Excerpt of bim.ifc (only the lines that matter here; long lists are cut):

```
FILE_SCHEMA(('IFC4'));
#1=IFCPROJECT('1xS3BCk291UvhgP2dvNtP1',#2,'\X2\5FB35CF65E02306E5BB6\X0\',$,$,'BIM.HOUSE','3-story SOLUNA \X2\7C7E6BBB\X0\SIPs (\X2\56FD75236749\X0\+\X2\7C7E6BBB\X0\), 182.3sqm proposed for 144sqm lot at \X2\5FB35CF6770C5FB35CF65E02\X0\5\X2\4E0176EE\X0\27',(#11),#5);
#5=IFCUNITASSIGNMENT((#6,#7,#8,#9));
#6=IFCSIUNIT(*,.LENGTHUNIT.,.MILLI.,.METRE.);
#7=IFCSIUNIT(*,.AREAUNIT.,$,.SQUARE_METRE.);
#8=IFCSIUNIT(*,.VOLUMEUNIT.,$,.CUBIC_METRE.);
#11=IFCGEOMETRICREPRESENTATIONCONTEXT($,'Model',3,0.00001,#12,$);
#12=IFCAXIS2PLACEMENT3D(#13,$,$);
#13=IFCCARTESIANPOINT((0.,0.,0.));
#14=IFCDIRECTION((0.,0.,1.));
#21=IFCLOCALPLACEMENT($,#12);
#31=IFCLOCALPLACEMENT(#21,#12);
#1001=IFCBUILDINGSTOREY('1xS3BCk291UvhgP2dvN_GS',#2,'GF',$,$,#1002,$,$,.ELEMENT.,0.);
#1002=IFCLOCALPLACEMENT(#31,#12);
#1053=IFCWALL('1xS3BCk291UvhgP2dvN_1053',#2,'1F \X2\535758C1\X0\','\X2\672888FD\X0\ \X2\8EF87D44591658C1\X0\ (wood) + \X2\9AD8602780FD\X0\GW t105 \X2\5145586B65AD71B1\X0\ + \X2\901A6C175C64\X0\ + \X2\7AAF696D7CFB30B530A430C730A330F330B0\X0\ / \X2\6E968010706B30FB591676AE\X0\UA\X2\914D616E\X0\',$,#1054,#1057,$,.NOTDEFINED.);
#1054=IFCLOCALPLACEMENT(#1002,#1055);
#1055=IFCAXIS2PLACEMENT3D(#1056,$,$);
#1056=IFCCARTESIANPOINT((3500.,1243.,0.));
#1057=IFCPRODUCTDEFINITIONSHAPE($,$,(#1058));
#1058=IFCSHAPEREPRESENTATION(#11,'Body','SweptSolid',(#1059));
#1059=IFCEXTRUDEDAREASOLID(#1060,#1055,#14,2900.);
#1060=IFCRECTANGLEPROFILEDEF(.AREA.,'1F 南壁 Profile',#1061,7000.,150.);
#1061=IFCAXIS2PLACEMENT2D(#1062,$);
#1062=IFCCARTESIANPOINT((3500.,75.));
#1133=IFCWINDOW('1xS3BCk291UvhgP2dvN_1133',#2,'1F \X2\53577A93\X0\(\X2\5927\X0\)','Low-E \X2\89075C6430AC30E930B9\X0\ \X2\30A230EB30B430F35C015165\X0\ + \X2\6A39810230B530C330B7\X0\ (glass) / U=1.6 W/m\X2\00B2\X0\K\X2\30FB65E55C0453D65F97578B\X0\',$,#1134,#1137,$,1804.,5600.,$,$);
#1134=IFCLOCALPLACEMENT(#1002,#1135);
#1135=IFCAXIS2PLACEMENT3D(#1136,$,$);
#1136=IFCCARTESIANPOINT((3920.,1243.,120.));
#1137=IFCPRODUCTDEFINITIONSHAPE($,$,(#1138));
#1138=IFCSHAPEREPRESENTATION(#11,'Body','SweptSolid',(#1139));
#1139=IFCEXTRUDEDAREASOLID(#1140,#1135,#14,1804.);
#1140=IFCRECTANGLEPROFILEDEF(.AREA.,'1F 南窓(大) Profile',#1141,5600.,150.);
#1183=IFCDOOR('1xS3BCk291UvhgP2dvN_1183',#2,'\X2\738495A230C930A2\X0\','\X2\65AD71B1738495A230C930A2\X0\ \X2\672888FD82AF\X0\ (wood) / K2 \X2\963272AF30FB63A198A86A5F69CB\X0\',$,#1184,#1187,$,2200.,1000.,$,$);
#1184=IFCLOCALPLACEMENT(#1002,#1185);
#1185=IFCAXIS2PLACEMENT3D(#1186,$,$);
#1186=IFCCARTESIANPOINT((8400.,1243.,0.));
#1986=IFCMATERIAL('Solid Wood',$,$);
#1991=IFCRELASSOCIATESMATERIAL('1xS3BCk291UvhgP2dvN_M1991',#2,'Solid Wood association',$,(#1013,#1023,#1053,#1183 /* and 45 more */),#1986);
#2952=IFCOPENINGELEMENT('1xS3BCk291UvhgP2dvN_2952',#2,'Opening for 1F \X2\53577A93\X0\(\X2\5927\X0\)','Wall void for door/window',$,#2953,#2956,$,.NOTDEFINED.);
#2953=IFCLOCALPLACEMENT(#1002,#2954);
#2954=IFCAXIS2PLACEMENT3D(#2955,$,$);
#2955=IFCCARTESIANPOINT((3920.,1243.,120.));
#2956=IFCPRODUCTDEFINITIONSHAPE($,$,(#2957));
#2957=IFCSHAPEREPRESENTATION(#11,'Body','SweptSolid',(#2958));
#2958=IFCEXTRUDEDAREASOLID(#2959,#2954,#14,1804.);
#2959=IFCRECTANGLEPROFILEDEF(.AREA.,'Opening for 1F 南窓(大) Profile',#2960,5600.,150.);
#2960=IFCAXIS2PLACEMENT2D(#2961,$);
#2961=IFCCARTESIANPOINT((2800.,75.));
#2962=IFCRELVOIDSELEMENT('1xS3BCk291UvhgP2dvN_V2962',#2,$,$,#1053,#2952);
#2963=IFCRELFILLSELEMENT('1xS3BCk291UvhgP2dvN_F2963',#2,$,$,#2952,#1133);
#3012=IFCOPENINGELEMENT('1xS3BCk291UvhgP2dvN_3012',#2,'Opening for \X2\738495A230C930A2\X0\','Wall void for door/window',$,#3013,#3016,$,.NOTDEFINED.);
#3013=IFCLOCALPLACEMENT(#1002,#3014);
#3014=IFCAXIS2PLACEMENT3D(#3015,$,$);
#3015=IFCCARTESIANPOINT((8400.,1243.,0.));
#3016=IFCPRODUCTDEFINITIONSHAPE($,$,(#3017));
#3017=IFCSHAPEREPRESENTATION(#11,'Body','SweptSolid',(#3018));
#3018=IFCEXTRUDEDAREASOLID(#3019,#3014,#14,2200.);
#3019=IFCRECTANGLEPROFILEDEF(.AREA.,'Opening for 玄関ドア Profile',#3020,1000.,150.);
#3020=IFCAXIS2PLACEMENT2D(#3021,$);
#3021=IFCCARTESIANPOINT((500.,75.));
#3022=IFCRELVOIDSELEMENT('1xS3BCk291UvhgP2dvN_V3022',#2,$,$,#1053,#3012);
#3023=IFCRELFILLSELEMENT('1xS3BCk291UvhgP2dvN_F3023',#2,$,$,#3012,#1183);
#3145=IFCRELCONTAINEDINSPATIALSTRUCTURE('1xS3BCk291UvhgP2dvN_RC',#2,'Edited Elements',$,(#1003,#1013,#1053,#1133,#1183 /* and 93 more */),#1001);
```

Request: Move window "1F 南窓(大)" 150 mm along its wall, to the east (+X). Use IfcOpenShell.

```python
import ifcopenshell
import ifcopenshell.api.geometry
import ifcopenshell.util.placement

model = ifcopenshell.open("bim.ifc")

window = model.by_guid("1xS3BCk291UvhgP2dvN_1133")
opening = window.FillsVoids[0].RelatingOpeningElement
wall = opening.VoidsElements[0].RelatingBuildingElement

wall_matrix = ifcopenshell.util.placement.get_local_placement(wall.ObjectPlacement)
shift = wall_matrix[:3, 0] * 150.0
before = ifcopenshell.util.placement.get_local_placement(window.ObjectPlacement)[:3, 3].copy()

# The window is not placed relative to its opening, so move both.
for product in (opening, window):
    matrix = ifcopenshell.util.placement.get_local_placement(product.ObjectPlacement)
    matrix[:3, 3] += shift
    ifcopenshell.api.geometry.edit_object_placement(model, product=product, matrix=matrix, is_si=False)

after = ifcopenshell.util.placement.get_local_placement(window.ObjectPlacement)[:3, 3]
print("window moved by", (after - before).round(3) + 0.0)

model.write("bim_updated.ifc")
```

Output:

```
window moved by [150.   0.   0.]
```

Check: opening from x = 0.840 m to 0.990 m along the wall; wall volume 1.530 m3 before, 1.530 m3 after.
